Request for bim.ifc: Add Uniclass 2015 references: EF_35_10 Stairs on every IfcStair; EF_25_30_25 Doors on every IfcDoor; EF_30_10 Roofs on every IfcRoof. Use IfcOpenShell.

First a look at what the model holds.

```python
import ifcopenshell

model = ifcopenshell.open("bim.ifc")
print(model.schema)
print("classifications:", [c.Name for c in model.by_type("IfcClassification")])
for ifc_class in ("IfcDoor", "IfcRoof", "IfcStair", "IfcWall", "IfcWindow"):
    print(ifc_class, len(model.by_type(ifc_class)))
```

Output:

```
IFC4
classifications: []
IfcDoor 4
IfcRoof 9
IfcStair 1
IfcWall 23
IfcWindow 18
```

```python
import ifcopenshell
import ifcopenshell.api.classification

model = ifcopenshell.open("bim.ifc")

system = ifcopenshell.api.classification.add_classification(model, classification="Uniclass 2015")

codes = {
    "IfcStair": ("EF_35_10", "Stairs"),
    "IfcDoor": ("EF_25_30_25", "Doors"),
    "IfcRoof": ("EF_30_10", "Roofs"),
}
for ifc_class, (code, name) in codes.items():
    products = model.by_type(ifc_class)
    ifcopenshell.api.classification.add_reference(
        model, products=products, classification=system, identification=code, name=name
    )
    print(code, len(products))

model.write("bim_updated.ifc")
```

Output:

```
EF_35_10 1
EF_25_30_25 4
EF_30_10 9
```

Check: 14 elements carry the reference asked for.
